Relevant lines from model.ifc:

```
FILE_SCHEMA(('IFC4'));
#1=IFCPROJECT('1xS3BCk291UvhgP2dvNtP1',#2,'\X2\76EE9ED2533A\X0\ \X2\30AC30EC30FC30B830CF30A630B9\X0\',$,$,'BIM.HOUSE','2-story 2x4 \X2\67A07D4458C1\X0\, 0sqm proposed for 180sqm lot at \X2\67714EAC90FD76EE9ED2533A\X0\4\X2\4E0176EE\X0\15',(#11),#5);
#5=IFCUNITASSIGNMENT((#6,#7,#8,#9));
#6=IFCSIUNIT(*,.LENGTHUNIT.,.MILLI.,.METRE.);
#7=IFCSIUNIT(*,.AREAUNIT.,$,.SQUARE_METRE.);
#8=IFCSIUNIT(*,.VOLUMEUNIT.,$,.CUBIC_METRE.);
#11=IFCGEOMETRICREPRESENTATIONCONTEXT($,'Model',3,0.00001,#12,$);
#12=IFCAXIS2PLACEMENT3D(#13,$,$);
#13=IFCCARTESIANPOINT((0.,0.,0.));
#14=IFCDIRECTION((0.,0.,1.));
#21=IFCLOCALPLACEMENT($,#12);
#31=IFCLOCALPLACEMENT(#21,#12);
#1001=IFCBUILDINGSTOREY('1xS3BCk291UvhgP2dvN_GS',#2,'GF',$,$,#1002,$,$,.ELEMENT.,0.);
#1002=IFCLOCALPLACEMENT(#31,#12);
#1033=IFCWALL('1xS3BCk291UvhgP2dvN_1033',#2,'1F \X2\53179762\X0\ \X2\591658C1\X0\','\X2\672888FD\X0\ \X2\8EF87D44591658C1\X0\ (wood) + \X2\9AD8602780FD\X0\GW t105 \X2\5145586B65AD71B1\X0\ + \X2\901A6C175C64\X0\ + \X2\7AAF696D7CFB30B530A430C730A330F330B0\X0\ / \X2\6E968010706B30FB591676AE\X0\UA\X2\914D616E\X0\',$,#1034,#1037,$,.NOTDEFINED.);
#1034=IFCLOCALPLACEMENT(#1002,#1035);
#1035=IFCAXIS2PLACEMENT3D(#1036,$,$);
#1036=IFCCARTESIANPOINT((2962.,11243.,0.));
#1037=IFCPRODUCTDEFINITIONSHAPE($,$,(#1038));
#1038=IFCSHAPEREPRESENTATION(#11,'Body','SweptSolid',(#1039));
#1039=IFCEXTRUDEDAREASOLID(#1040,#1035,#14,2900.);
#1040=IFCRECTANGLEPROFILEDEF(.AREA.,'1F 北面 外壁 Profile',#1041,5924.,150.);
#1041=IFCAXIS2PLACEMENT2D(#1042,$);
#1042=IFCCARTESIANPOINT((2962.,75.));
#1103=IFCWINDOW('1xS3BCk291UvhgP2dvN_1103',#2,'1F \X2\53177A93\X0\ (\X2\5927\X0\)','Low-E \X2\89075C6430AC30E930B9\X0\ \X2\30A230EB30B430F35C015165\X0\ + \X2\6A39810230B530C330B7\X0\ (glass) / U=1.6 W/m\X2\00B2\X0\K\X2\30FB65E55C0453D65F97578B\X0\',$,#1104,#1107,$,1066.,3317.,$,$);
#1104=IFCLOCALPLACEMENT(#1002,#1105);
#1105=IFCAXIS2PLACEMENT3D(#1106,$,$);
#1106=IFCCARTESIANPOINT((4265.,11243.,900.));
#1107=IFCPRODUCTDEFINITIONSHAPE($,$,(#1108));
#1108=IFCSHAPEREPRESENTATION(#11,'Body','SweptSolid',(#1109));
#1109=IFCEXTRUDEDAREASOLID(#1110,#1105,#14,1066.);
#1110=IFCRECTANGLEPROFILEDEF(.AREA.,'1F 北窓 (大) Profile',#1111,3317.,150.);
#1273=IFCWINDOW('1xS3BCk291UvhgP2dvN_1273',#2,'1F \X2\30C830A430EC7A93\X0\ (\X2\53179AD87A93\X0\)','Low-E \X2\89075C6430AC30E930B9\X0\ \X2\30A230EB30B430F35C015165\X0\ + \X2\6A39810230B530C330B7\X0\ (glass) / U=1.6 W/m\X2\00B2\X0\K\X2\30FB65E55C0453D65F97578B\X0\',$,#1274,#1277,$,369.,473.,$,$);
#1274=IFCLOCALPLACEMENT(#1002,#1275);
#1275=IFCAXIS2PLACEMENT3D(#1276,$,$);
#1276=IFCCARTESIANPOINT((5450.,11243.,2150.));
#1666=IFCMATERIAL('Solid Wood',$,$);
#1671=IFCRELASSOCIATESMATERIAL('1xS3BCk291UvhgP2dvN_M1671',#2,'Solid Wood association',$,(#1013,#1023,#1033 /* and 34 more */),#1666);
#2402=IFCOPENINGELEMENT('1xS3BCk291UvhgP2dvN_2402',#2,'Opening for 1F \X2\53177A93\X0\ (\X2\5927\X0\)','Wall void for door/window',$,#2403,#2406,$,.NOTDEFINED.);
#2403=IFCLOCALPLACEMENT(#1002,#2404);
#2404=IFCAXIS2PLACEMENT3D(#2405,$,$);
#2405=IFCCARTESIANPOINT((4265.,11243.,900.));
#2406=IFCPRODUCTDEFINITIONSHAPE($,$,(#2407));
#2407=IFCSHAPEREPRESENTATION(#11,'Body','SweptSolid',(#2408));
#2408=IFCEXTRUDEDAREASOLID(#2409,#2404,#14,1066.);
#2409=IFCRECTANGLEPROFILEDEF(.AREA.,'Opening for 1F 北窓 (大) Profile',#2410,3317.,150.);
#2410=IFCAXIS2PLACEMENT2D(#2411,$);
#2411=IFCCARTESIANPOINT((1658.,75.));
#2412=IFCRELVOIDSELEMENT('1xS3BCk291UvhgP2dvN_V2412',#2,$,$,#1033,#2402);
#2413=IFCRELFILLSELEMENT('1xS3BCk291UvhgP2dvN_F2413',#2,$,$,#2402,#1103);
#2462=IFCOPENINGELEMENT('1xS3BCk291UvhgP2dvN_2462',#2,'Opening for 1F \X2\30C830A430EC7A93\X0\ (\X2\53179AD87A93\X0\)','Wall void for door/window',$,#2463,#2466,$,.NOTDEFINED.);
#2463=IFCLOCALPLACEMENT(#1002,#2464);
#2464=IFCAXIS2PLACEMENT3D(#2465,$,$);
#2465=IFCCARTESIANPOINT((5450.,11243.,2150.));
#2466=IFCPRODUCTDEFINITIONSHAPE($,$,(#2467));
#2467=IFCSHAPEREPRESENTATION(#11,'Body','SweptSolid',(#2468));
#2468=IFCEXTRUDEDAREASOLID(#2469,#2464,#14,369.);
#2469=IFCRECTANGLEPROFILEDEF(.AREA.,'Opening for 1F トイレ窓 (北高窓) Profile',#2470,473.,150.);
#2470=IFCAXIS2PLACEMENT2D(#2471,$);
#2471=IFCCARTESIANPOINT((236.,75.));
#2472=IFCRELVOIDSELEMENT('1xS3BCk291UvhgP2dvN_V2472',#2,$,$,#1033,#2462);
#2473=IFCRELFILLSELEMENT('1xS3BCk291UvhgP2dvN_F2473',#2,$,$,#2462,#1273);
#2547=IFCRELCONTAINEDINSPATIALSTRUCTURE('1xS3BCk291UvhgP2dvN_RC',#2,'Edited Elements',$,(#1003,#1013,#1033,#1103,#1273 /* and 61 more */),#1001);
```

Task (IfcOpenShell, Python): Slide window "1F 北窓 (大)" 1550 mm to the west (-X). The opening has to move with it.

```python
import ifcopenshell
import ifcopenshell.api.geometry
import ifcopenshell.util.placement
import ifcopenshell.util.unit

model = ifcopenshell.open("model.ifc")
unit_scale = ifcopenshell.util.unit.calculate_unit_scale(model)

window = model.by_id(1103)
opening = window.FillsVoids[0].RelatingOpeningElement
wall = opening.VoidsElements[0].RelatingBuildingElement

wall_matrix = ifcopenshell.util.placement.get_local_placement(wall.ObjectPlacement)
shift = wall_matrix[:3, 0] * -1.55 / unit_scale
before = ifcopenshell.util.placement.get_local_placement(window.ObjectPlacement)[:3, 3].copy()

# The window is not placed relative to its opening, so move both.
for product in (opening, window):
    matrix = ifcopenshell.util.placement.get_local_placement(product.ObjectPlacement)
    matrix[:3, 3] += shift
    ifcopenshell.api.geometry.edit_object_placement(model, product=product, matrix=matrix, is_si=False)

after = ifcopenshell.util.placement.get_local_placement(window.ObjectPlacement)[:3, 3]
print("window moved by", (after - before).round(3) + 0.0)

model.write("model-out.ifc")
```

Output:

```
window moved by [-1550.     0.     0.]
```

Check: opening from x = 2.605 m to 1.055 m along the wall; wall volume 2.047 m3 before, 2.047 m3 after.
